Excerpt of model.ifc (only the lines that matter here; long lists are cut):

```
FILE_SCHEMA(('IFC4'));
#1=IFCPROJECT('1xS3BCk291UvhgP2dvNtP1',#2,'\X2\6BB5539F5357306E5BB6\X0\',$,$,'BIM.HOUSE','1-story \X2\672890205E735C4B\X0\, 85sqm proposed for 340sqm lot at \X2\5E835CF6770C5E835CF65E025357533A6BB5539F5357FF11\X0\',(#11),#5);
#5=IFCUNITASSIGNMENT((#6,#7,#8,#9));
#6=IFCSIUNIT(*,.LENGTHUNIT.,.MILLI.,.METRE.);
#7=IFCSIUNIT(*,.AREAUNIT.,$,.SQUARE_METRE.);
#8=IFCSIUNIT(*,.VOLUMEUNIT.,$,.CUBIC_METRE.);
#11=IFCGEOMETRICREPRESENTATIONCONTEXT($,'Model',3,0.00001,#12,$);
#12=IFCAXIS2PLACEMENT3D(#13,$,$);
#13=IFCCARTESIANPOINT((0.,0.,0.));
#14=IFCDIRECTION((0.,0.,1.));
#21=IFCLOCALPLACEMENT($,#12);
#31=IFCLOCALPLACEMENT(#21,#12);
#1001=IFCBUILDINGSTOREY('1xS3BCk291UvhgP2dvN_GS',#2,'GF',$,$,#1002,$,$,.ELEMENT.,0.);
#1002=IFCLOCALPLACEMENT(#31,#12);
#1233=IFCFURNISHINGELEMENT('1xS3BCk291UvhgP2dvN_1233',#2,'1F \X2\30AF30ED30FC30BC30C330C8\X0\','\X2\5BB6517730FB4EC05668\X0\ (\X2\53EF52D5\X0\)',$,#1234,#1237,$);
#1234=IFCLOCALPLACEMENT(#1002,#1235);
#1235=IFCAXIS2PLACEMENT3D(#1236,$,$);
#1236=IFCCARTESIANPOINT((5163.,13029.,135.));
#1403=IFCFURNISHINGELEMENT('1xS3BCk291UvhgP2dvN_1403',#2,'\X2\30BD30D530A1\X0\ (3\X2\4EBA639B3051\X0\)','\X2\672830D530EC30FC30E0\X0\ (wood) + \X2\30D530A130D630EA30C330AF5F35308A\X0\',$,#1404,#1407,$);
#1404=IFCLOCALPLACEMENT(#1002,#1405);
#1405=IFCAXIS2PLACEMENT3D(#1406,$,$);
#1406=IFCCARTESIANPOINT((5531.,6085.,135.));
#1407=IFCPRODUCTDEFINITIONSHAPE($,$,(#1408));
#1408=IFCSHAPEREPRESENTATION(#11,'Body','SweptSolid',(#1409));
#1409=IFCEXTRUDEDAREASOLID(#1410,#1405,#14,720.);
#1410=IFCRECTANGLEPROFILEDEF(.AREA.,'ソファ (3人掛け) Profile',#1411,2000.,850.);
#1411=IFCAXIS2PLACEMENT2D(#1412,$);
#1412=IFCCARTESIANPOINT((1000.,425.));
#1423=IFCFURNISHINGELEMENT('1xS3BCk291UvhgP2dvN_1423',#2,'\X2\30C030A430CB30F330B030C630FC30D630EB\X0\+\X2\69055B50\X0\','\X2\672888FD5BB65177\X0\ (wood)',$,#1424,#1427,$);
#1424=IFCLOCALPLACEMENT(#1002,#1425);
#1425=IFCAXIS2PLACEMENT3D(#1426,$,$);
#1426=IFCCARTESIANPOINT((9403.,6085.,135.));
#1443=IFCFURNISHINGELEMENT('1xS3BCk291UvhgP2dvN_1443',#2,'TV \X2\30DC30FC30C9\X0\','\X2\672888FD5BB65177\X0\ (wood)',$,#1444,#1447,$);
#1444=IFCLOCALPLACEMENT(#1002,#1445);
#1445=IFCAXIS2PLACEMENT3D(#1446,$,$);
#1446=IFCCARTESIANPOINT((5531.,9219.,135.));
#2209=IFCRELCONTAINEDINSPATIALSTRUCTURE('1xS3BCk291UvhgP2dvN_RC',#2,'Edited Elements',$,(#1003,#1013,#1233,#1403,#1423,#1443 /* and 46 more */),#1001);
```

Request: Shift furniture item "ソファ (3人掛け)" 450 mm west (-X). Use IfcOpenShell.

```python
import ifcopenshell
import ifcopenshell.api.geometry
import ifcopenshell.util.placement

model = ifcopenshell.open("model.ifc")

item = model.by_guid("1xS3BCk291UvhgP2dvN_1403")
matrix = ifcopenshell.util.placement.get_local_placement(item.ObjectPlacement)
matrix[0, 3] -= 450.0
ifcopenshell.api.geometry.edit_object_placement(model, product=item, matrix=matrix, is_si=False)

print(ifcopenshell.util.placement.get_local_placement(item.ObjectPlacement).round(3) + 0.0)

model.write("model_updated.ifc")
```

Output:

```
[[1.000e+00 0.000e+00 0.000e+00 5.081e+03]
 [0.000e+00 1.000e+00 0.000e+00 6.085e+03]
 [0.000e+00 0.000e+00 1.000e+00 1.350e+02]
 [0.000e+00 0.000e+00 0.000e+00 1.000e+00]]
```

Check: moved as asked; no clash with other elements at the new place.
